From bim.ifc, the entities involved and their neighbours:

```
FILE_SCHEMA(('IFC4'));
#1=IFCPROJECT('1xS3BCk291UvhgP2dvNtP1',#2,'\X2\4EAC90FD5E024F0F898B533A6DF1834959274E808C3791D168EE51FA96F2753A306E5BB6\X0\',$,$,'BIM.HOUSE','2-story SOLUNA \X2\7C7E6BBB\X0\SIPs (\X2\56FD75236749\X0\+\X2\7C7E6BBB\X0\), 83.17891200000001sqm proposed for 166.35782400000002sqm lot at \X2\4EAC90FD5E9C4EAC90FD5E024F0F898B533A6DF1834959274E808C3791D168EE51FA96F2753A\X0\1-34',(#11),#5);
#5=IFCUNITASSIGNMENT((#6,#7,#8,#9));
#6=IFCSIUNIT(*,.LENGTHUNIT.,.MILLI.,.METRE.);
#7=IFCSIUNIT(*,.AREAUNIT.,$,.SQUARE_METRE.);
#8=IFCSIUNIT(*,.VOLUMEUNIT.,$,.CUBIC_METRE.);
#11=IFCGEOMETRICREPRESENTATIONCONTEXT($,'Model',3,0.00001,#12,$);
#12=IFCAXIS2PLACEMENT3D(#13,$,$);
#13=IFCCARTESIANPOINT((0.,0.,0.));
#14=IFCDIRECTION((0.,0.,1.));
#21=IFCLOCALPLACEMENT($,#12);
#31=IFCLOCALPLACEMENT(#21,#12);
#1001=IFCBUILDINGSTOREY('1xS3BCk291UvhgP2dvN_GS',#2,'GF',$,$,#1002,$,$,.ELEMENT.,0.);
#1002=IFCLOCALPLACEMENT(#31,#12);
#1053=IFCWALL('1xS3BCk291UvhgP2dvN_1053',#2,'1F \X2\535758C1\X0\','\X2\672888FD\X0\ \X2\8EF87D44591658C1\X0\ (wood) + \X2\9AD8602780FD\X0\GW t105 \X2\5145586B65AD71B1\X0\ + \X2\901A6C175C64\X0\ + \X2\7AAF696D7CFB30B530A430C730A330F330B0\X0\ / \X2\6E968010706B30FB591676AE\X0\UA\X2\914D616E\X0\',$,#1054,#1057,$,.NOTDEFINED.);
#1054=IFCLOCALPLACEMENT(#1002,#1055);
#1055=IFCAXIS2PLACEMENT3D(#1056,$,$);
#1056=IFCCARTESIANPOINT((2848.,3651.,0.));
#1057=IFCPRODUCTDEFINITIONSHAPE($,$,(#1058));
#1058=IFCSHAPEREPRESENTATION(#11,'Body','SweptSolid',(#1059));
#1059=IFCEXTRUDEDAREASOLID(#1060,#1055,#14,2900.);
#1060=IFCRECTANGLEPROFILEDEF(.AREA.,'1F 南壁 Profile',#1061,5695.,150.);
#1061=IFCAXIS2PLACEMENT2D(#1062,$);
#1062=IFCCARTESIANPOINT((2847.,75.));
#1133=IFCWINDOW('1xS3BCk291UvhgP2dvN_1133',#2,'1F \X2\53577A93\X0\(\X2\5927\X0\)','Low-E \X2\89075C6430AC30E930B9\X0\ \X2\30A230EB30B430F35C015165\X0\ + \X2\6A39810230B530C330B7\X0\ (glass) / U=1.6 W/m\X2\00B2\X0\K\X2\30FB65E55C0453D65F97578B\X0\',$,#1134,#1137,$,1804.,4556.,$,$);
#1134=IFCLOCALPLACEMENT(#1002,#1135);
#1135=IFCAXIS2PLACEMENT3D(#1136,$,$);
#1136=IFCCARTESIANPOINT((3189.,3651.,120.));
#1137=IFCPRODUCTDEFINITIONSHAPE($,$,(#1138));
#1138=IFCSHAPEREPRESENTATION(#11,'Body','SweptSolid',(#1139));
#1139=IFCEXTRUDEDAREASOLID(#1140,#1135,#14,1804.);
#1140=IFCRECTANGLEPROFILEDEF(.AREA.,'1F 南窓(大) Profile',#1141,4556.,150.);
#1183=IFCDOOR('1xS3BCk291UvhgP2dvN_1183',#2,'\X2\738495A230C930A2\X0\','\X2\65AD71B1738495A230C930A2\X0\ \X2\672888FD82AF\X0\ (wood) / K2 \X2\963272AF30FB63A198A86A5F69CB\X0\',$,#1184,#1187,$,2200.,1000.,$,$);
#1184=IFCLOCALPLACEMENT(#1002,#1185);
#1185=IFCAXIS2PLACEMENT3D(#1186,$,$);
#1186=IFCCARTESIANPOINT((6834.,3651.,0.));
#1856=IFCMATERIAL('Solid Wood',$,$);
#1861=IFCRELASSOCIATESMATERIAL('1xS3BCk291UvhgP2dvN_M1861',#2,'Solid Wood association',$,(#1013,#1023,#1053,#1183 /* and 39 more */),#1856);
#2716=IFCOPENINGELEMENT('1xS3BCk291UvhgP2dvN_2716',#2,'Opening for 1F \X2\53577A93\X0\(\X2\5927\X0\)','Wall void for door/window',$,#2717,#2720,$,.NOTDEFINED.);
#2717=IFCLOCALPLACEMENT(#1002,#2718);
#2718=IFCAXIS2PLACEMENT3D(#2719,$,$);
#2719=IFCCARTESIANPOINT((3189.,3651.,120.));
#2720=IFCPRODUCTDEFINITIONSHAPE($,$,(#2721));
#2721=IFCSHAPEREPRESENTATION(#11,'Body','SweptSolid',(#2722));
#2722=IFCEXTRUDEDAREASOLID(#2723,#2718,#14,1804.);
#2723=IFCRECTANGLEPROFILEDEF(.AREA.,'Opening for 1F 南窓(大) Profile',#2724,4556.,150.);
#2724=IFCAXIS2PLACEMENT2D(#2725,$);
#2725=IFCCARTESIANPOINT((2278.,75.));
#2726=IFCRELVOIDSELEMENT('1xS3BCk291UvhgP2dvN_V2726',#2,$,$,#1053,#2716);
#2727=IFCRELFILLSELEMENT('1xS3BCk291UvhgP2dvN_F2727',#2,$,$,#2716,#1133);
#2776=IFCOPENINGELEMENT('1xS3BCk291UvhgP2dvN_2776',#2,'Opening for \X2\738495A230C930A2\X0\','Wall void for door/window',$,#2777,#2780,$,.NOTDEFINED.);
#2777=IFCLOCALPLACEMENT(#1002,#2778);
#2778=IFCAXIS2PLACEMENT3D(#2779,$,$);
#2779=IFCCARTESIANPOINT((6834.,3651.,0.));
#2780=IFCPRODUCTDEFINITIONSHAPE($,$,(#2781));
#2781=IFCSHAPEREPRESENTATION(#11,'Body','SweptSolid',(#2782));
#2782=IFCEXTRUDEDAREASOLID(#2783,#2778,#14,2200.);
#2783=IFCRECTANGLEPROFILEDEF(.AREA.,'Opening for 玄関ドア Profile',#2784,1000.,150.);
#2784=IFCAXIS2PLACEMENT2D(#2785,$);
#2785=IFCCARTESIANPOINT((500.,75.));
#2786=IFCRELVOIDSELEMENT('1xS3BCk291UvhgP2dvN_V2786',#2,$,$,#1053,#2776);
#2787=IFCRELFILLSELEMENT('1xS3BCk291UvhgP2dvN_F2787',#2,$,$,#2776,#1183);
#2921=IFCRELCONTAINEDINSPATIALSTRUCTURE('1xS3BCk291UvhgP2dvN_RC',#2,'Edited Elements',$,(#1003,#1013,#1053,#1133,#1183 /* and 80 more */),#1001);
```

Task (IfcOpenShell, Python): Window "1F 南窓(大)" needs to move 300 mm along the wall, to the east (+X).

```python
import ifcopenshell
import ifcopenshell.api.geometry
import ifcopenshell.util.placement
import ifcopenshell.util.unit

model = ifcopenshell.open("bim.ifc")
unit_scale = ifcopenshell.util.unit.calculate_unit_scale(model)

window = model.by_guid("1xS3BCk291UvhgP2dvN_1133")
opening = window.FillsVoids[0].RelatingOpeningElement
wall = opening.VoidsElements[0].RelatingBuildingElement

wall_matrix = ifcopenshell.util.placement.get_local_placement(wall.ObjectPlacement)
shift = wall_matrix[:3, 0] * 0.3 / unit_scale
before = ifcopenshell.util.placement.get_local_placement(window.ObjectPlacement)[:3, 3].copy()

# The window is not placed relative to its opening, so move both.
for product in (opening, window):
    matrix = ifcopenshell.util.placement.get_local_placement(product.ObjectPlacement)
    matrix[:3, 3] += shift
    ifcopenshell.api.geometry.edit_object_placement(model, product=product, matrix=matrix, is_si=False)

after = ifcopenshell.util.placement.get_local_placement(window.ObjectPlacement)[:3, 3]
print("window moved by", (after - before).round(3) + 0.0)

model.write("bim_updated.ifc")
```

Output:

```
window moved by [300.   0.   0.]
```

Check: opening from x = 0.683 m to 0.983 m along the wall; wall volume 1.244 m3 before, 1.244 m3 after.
